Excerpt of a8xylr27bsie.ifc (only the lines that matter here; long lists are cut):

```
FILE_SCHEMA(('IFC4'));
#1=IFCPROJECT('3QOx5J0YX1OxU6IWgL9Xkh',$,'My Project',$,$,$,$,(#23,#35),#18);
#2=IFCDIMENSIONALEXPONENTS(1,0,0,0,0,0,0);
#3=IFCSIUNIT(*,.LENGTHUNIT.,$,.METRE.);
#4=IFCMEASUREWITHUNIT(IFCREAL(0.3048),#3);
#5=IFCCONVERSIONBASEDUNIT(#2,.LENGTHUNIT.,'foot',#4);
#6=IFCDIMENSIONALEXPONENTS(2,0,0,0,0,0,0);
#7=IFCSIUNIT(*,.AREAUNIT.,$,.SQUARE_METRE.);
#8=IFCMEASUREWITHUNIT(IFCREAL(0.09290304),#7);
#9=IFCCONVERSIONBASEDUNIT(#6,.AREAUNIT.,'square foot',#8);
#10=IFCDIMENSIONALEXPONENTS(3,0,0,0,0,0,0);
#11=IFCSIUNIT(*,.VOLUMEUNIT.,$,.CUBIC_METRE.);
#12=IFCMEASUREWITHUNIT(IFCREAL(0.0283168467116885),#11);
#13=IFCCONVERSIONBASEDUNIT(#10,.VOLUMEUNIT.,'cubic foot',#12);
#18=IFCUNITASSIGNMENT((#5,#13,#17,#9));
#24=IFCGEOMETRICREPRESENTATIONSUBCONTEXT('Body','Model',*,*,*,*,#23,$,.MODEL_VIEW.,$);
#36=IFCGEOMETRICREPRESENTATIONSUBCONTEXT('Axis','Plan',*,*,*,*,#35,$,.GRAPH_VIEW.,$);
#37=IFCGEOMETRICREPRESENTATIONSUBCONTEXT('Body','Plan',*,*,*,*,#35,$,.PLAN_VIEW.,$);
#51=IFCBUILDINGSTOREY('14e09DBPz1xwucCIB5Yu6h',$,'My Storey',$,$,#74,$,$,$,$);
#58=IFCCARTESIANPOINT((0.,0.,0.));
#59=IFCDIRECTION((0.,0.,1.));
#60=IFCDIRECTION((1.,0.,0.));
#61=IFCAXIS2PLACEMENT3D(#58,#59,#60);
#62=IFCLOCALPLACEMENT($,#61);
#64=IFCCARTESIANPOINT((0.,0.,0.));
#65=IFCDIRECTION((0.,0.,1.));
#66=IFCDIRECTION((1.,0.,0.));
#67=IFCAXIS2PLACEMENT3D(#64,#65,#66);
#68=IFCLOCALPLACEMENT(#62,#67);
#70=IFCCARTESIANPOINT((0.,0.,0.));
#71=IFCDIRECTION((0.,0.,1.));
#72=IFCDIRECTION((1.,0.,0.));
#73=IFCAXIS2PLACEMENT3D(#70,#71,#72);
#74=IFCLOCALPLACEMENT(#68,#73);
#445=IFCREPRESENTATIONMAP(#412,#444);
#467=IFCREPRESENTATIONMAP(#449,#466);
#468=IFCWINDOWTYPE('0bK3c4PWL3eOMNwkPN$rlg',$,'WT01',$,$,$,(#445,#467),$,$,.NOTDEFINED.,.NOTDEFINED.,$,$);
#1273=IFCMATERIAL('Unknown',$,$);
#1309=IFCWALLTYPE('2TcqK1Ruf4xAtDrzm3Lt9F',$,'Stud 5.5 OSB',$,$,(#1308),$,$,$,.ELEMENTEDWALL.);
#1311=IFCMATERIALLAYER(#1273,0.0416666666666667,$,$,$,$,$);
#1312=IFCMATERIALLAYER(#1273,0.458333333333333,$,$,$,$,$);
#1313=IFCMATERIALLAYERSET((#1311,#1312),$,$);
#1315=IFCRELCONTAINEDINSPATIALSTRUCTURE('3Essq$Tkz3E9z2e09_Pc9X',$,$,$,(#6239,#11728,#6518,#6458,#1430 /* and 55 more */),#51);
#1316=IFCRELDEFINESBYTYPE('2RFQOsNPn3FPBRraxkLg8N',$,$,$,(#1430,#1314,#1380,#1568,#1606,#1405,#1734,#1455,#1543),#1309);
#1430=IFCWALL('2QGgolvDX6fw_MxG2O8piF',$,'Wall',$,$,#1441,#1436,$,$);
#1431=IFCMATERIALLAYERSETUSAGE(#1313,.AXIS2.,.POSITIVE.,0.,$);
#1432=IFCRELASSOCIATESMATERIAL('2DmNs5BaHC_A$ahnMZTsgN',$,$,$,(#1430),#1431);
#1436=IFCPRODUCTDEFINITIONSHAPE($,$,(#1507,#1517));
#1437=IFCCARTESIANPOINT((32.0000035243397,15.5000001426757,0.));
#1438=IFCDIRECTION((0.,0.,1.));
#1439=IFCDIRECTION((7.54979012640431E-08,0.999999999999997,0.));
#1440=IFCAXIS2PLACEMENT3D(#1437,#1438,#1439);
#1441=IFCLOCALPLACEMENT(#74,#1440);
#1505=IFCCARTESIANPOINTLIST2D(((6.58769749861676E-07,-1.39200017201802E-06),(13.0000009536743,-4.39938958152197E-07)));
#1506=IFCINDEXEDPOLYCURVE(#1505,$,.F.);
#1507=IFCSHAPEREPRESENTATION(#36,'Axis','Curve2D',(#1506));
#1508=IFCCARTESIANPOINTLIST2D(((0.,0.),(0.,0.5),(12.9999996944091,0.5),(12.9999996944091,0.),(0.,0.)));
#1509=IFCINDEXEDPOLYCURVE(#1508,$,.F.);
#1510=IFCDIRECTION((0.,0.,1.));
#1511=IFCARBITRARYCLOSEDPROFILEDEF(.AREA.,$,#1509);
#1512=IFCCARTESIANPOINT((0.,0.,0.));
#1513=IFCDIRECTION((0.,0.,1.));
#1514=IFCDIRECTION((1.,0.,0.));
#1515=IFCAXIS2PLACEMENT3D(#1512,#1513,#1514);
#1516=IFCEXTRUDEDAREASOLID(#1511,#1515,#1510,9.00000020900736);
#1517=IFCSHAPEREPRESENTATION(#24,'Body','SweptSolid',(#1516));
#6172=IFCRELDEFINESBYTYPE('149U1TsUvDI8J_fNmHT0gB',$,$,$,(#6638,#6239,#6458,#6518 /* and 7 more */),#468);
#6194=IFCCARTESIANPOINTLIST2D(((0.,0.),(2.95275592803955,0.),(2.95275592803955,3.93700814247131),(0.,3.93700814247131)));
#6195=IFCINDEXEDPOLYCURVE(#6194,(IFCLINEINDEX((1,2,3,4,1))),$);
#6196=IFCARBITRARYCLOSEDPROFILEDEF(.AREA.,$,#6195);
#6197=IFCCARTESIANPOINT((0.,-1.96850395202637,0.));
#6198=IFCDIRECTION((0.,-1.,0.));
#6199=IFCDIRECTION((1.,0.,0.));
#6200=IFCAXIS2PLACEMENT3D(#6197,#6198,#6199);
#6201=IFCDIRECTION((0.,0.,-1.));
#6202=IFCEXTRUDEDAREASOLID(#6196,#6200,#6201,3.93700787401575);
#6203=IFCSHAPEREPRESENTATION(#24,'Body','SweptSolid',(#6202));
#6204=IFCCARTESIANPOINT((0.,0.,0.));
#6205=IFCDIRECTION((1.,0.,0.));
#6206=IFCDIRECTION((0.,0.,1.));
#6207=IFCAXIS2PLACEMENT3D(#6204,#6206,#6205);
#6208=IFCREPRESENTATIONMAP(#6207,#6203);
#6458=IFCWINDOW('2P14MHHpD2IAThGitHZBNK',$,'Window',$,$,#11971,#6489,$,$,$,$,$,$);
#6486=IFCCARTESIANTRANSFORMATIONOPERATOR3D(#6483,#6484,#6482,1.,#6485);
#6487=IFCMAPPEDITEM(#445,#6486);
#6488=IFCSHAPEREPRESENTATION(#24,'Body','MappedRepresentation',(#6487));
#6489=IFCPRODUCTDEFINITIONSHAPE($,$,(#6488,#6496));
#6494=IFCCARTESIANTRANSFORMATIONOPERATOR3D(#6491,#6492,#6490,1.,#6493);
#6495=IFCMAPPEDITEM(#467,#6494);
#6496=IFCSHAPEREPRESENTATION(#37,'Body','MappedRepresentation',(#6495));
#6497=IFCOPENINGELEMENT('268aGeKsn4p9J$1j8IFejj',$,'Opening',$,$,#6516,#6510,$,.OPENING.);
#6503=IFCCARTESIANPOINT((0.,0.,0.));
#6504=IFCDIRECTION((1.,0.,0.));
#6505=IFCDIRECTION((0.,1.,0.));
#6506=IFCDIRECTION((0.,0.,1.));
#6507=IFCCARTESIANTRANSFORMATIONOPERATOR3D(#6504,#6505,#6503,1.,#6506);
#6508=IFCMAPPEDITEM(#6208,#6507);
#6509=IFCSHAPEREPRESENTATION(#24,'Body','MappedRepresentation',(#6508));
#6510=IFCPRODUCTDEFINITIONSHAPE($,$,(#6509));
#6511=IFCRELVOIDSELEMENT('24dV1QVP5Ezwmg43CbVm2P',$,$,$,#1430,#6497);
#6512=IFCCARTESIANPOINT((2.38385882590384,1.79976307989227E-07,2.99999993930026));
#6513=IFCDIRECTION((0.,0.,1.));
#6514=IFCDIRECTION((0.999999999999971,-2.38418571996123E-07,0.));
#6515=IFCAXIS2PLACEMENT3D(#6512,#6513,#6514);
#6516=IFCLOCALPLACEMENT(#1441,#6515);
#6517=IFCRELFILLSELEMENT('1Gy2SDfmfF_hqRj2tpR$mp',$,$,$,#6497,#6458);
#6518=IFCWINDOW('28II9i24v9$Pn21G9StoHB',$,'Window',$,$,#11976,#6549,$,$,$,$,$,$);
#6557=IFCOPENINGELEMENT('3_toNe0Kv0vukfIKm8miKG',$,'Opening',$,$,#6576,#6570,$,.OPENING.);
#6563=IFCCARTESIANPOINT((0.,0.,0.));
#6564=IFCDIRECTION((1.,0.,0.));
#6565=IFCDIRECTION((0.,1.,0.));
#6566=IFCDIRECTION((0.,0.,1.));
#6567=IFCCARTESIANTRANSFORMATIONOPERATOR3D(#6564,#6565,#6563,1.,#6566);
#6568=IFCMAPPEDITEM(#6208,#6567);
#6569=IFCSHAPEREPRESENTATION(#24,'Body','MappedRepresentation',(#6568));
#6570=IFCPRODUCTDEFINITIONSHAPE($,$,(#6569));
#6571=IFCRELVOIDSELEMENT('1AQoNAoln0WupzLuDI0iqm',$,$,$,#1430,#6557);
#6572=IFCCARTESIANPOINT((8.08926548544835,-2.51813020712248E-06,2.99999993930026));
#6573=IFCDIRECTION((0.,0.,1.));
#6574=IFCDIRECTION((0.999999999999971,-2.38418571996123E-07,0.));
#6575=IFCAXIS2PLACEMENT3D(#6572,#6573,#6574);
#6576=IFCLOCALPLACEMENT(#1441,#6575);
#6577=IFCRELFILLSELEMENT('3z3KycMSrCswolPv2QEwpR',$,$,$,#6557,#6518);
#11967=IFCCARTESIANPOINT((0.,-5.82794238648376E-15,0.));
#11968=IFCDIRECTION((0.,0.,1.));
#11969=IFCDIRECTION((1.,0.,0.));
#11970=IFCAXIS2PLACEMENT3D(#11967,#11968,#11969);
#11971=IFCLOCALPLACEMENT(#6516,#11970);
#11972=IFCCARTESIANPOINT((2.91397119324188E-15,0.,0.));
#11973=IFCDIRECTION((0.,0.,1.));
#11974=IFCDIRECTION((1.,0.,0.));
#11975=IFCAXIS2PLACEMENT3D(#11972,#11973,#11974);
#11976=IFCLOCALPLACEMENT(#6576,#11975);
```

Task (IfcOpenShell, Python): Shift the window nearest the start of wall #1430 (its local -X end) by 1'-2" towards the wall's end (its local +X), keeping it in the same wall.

```python
import ifcopenshell
import ifcopenshell.api.geometry
import ifcopenshell.util.placement
import ifcopenshell.util.unit

model = ifcopenshell.open("a8xylr27bsie.ifc")
unit_scale = ifcopenshell.util.unit.calculate_unit_scale(model)

window = model.by_id(6458)
opening = window.FillsVoids[0].RelatingOpeningElement
wall = opening.VoidsElements[0].RelatingBuildingElement

wall_matrix = ifcopenshell.util.placement.get_local_placement(wall.ObjectPlacement)
shift = wall_matrix[:3, 0] * 14 * 0.0254 / unit_scale
before = ifcopenshell.util.placement.get_local_placement(window.ObjectPlacement)[:3, 3].copy()

# The window is placed relative to its opening, so it follows when the opening moves.
matrix = ifcopenshell.util.placement.get_local_placement(opening.ObjectPlacement)
matrix[:3, 3] += shift
ifcopenshell.api.geometry.edit_object_placement(
    model, product=opening, matrix=matrix, is_si=False, should_transform_children=True
)

after = ifcopenshell.util.placement.get_local_placement(window.ObjectPlacement)[:3, 3]
print("window moved by", (after - before).round(3) + 0.0)

model.write("a8xylr27bsie-out.ifc")
```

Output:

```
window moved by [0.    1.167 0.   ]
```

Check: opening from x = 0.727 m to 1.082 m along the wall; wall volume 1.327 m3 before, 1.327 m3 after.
